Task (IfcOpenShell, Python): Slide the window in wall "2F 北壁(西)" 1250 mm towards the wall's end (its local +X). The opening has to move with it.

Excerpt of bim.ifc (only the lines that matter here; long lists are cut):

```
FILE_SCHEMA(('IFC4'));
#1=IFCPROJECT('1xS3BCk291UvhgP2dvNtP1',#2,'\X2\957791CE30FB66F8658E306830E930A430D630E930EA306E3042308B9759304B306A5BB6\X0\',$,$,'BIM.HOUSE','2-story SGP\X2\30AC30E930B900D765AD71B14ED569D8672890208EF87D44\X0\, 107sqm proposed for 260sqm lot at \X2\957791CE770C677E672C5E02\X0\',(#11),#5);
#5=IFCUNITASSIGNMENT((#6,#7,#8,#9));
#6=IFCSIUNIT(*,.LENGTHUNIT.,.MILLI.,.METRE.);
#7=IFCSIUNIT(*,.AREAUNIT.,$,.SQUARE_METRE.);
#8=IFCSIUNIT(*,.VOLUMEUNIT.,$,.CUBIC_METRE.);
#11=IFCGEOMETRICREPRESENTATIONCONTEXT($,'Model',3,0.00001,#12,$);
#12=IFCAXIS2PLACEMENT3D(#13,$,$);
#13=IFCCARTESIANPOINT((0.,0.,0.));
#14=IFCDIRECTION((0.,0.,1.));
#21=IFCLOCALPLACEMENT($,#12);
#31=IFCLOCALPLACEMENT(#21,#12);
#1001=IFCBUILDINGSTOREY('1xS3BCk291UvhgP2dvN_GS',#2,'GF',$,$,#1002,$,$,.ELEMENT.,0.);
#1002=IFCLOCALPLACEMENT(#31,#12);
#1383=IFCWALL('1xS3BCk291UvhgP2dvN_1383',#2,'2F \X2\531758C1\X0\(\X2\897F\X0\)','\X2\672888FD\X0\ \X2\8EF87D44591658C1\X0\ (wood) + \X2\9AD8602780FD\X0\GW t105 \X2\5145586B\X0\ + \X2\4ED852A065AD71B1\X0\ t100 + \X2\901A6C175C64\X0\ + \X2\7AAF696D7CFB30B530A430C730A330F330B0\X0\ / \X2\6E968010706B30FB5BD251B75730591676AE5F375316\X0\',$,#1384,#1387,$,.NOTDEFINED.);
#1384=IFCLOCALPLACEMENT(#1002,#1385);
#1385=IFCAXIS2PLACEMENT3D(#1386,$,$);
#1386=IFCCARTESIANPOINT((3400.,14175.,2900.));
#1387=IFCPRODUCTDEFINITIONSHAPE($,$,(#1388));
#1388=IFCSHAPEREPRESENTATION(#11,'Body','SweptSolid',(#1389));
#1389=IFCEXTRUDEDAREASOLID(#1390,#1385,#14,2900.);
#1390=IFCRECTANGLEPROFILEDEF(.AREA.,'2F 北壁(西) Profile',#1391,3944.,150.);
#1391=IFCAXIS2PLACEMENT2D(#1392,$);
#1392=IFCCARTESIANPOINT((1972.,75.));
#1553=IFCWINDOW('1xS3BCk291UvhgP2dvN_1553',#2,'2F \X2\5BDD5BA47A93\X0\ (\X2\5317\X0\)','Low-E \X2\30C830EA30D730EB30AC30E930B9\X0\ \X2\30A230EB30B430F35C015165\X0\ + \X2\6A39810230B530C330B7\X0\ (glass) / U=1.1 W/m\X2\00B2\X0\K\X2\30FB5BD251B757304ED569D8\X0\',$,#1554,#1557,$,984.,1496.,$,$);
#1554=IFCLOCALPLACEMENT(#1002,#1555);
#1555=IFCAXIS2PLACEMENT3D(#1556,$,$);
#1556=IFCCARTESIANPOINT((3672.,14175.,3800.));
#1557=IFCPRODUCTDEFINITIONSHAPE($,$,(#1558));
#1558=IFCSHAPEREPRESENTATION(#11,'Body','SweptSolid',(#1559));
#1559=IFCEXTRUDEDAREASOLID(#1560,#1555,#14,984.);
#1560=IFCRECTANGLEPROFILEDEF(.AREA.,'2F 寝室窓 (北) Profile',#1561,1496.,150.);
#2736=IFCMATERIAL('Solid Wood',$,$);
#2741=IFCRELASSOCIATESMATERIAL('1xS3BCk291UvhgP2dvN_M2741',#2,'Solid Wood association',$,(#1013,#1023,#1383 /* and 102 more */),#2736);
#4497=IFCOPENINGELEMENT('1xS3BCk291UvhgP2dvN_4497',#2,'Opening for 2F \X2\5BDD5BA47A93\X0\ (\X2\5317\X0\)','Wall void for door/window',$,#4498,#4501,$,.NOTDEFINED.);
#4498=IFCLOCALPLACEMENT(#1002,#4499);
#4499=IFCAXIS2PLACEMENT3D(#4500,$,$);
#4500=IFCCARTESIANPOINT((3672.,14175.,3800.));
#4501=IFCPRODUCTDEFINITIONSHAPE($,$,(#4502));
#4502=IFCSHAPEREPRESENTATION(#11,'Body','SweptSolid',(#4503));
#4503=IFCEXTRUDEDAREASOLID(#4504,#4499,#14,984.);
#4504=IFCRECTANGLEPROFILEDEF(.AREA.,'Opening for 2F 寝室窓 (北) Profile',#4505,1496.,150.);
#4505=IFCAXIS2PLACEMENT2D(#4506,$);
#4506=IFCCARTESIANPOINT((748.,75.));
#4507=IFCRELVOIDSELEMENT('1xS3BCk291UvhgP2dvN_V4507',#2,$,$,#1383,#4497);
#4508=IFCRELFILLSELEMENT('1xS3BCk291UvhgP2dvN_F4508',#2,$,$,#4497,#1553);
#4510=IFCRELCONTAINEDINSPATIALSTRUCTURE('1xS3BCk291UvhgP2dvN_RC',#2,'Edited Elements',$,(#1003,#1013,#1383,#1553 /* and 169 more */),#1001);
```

```python
import ifcopenshell
import ifcopenshell.api.geometry
import ifcopenshell.util.placement
import ifcopenshell.util.unit

model = ifcopenshell.open("bim.ifc")
unit_scale = ifcopenshell.util.unit.calculate_unit_scale(model)

window = model.by_guid("1xS3BCk291UvhgP2dvN_1553")
opening = window.FillsVoids[0].RelatingOpeningElement
wall = opening.VoidsElements[0].RelatingBuildingElement

wall_matrix = ifcopenshell.util.placement.get_local_placement(wall.ObjectPlacement)
shift = wall_matrix[:3, 0] * 1.25 / unit_scale
before = ifcopenshell.util.placement.get_local_placement(window.ObjectPlacement)[:3, 3].copy()

# The window is not placed relative to its opening, so move both.
for product in (opening, window):
    matrix = ifcopenshell.util.placement.get_local_placement(product.ObjectPlacement)
    matrix[:3, 3] += shift
    ifcopenshell.api.geometry.edit_object_placement(model, product=product, matrix=matrix, is_si=False)

after = ifcopenshell.util.placement.get_local_placement(window.ObjectPlacement)[:3, 3]
print("window moved by", (after - before).round(3) + 0.0)

model.write("bim_rev.ifc")
```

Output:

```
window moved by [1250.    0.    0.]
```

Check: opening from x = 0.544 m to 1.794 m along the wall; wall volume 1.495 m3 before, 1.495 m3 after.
